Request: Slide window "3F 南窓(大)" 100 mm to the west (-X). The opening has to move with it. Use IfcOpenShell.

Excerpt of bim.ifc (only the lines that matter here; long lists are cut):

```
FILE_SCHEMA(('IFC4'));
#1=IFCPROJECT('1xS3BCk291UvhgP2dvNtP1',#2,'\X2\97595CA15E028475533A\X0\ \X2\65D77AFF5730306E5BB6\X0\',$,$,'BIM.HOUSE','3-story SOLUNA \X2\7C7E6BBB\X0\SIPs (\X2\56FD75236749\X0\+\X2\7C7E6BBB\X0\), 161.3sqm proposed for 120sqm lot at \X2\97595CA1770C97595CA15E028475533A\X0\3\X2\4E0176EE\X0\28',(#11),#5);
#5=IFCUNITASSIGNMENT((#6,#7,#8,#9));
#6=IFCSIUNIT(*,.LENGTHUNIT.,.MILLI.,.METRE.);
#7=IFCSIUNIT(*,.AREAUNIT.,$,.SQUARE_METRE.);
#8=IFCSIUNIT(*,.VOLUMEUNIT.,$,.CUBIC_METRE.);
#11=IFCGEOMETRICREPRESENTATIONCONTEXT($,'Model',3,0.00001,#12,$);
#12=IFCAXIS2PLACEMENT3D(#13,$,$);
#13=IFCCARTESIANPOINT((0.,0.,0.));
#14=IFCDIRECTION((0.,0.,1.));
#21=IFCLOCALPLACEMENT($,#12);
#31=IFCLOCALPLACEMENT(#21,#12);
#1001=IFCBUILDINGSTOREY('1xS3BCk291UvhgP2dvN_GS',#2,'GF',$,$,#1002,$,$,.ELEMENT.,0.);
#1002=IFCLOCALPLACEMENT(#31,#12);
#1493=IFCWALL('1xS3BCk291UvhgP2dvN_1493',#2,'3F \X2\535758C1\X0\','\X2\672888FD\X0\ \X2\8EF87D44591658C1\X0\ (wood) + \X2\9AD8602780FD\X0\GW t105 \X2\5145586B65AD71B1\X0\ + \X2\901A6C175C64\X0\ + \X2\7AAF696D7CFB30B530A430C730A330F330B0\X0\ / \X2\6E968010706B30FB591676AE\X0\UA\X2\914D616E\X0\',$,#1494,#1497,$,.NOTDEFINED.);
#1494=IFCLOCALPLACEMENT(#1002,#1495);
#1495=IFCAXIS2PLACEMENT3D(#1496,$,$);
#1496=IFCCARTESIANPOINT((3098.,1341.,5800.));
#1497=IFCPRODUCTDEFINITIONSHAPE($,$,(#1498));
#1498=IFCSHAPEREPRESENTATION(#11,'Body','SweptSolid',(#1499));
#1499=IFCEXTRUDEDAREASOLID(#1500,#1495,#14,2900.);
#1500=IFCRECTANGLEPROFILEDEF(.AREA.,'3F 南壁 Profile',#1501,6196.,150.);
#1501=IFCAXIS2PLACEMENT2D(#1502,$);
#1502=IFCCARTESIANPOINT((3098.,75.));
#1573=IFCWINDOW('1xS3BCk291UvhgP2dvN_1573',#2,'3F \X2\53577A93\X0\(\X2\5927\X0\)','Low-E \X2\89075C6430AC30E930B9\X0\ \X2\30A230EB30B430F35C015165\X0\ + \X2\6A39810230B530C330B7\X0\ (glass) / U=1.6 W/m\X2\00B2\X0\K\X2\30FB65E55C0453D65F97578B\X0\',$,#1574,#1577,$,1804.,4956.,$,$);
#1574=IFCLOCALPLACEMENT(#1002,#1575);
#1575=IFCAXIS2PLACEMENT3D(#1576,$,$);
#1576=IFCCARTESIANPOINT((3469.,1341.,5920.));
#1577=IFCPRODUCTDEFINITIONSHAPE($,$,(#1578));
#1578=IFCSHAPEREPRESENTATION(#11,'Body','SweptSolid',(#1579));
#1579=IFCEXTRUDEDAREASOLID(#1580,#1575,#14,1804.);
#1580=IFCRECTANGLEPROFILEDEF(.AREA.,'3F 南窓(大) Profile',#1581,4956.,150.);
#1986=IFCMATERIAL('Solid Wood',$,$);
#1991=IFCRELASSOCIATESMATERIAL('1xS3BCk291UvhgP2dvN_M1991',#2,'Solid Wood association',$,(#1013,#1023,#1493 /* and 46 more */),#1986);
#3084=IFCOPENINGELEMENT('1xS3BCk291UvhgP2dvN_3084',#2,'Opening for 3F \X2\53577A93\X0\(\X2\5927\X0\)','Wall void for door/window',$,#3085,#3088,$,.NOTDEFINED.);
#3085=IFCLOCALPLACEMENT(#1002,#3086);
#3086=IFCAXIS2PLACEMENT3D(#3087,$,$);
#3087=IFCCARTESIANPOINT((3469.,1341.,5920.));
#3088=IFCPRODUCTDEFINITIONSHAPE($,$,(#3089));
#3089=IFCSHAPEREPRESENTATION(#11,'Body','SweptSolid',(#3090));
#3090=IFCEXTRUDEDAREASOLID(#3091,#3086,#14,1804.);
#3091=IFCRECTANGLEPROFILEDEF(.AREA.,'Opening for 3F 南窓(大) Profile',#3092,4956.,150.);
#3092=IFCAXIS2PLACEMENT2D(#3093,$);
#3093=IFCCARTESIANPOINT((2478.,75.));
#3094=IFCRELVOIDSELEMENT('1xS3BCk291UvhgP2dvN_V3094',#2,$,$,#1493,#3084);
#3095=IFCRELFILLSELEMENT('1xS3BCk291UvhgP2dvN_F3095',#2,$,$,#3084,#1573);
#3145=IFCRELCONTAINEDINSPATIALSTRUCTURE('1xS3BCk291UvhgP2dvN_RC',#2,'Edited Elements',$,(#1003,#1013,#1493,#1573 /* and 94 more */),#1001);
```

```python
import ifcopenshell
import ifcopenshell.api.geometry
import ifcopenshell.util.placement
import ifcopenshell.util.unit

model = ifcopenshell.open("bim.ifc")
unit_scale = ifcopenshell.util.unit.calculate_unit_scale(model)

window = model.by_guid("1xS3BCk291UvhgP2dvN_1573")
opening = window.FillsVoids[0].RelatingOpeningElement
wall = opening.VoidsElements[0].RelatingBuildingElement

wall_matrix = ifcopenshell.util.placement.get_local_placement(wall.ObjectPlacement)
shift = wall_matrix[:3, 0] * -0.1 / unit_scale
before = ifcopenshell.util.placement.get_local_placement(window.ObjectPlacement)[:3, 3].copy()

# The window is not placed relative to its opening, so move both.
for product in (opening, window):
    matrix = ifcopenshell.util.placement.get_local_placement(product.ObjectPlacement)
    matrix[:3, 3] += shift
    ifcopenshell.api.geometry.edit_object_placement(model, product=product, matrix=matrix, is_si=False)

after = ifcopenshell.util.placement.get_local_placement(window.ObjectPlacement)[:3, 3]
print("window moved by", (after - before).round(3) + 0.0)

model.write("bim_edited.ifc")
```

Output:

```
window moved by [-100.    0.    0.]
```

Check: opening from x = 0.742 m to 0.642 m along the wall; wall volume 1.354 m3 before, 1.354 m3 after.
